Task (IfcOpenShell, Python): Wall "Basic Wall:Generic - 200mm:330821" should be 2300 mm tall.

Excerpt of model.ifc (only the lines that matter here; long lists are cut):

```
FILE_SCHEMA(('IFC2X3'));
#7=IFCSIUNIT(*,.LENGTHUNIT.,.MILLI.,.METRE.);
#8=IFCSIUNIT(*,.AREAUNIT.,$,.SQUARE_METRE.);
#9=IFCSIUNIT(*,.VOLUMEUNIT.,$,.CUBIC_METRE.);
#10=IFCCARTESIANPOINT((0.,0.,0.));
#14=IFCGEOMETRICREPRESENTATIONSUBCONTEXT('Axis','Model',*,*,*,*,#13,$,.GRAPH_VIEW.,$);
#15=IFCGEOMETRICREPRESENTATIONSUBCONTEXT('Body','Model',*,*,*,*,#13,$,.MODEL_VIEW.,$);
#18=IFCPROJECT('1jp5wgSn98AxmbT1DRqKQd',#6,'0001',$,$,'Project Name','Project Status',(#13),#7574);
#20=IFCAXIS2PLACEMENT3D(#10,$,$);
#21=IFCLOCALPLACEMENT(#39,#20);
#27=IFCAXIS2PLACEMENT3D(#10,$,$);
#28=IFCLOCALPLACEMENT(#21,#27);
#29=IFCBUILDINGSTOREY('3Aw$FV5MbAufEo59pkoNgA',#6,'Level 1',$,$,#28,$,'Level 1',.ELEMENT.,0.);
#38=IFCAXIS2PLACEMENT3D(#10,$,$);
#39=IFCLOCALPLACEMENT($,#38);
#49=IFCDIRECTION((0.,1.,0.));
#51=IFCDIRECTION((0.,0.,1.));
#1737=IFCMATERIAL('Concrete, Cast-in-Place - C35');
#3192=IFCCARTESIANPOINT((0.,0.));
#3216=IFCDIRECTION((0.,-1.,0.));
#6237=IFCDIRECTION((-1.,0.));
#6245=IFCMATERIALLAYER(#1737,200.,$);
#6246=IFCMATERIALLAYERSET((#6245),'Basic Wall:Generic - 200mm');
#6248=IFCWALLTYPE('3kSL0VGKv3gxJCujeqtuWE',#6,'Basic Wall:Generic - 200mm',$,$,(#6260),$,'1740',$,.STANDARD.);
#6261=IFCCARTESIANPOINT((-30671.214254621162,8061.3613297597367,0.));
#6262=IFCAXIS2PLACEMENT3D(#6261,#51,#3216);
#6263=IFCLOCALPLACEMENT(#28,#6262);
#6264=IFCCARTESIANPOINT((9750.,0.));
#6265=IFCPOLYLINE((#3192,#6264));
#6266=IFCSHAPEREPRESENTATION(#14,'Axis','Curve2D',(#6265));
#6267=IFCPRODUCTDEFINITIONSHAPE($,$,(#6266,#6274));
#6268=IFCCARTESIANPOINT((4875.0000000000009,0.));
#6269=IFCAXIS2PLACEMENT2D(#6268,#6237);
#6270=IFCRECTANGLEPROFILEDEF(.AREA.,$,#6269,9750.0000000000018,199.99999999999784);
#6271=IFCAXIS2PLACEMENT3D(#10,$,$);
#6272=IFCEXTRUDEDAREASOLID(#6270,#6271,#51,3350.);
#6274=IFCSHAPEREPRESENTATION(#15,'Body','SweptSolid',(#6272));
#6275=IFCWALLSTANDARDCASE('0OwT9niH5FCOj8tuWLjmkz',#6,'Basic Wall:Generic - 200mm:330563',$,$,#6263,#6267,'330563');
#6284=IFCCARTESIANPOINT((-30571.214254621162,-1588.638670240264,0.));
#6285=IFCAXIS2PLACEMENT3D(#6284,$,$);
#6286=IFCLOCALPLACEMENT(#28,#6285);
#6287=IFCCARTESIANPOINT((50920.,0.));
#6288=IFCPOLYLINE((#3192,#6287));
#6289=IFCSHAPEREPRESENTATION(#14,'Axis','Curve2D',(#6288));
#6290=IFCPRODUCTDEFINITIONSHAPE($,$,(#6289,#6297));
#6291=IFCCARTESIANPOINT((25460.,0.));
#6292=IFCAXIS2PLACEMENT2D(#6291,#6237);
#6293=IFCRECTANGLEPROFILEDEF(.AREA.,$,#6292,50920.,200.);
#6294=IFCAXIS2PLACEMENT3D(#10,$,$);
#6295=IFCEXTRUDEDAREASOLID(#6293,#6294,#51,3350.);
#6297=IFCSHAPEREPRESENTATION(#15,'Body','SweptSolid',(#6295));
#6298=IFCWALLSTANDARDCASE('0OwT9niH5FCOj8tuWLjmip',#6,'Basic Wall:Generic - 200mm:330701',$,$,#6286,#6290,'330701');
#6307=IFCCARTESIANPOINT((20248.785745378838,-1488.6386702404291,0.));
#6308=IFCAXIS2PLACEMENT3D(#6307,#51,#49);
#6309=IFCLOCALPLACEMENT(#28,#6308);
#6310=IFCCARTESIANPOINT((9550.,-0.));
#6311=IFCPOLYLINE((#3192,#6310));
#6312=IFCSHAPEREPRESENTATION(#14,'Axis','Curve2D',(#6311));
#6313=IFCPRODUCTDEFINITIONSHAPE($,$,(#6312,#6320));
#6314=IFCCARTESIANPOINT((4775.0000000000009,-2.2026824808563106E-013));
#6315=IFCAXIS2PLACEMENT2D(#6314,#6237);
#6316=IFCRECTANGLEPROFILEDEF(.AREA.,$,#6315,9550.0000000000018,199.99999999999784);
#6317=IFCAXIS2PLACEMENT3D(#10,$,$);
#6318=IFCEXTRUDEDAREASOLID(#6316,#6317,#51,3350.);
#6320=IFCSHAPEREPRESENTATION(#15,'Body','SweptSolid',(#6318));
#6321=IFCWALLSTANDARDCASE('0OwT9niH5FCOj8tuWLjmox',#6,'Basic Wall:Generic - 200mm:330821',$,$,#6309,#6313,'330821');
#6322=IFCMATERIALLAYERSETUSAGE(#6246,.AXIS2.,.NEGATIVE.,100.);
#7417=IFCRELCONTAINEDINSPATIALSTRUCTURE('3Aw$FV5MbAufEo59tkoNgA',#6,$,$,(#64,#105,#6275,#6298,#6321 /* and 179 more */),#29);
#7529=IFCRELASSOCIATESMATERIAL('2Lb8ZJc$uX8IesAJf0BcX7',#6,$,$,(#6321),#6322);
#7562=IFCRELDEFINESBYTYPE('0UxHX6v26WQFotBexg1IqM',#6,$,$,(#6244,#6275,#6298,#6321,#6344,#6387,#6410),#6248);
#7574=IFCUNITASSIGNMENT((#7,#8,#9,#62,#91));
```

```python
import ifcopenshell
import ifcopenshell.geom
import ifcopenshell.util.representation
import ifcopenshell.util.shape

model = ifcopenshell.open("model.ifc")
settings = ifcopenshell.geom.settings()


def volume(element):
    """Net volume in cubic metres, openings subtracted."""
    shape = ifcopenshell.geom.create_shape(settings, element)
    return ifcopenshell.util.shape.get_volume(shape.geometry)


wall = model.by_id(6321)
before = volume(wall)

body = ifcopenshell.util.representation.get_representation(wall, "Model", "Body")
solid = body.Items[0]
old_height = solid.Depth
solid.Depth = 2300.0
after = volume(wall)

print(f"height {old_height:g} -> {solid.Depth:g}, volume {before:.3f} -> {after:.3f} m3")

model.write("model_rev.ifc")
```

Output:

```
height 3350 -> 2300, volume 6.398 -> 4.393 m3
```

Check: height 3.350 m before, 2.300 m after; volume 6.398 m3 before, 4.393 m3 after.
